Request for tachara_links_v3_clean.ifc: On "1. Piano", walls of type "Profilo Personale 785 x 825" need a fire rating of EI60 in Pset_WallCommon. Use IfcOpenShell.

First a look at what the model holds.

```python
import ifcopenshell
import ifcopenshell.util.element

model = ifcopenshell.open("tachara_links_v3_clean.ifc")
print(model.schema)
storey = next(s for s in model.by_type("IfcBuildingStorey") if s.Name == "1. Piano")
walls = [e for e in ifcopenshell.util.element.get_decomposition(storey) if e.is_a("IfcWall")]
seen = {}
for e in walls:
    element_type = ifcopenshell.util.element.get_type(e)
    key = (element_type.Name if element_type != e and element_type else None, ifcopenshell.util.element.get_pset(e, "Pset_WallCommon", "FireRating"))
    seen[key] = seen.get(key, 0) + 1
for (name, value), count in sorted(seen.items(), key=str):
    print(count, "x", name, "|", value)
```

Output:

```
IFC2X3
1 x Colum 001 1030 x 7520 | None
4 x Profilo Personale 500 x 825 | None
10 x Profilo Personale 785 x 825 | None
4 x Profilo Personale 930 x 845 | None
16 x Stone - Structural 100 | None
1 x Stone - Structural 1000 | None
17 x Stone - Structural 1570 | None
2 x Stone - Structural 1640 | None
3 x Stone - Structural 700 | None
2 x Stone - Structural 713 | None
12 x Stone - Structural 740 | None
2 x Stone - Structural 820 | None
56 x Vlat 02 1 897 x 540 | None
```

```python
import ifcopenshell
import ifcopenshell.api.pset
import ifcopenshell.util.element

model = ifcopenshell.open("tachara_links_v3_clean.ifc")

storey = next(s for s in model.by_type("IfcBuildingStorey") if s.Name == "1. Piano")
walls = [e for e in ifcopenshell.util.element.get_decomposition(storey) if e.is_a("IfcWall")]

count = 0
for e in walls:
    element_type = ifcopenshell.util.element.get_type(e)
    if element_type in (None, e) or element_type.Name != "Profilo Personale 785 x 825":
        continue
    # add_pset returns the element's existing set when there is one.
    pset = ifcopenshell.api.pset.add_pset(model, product=e, name="Pset_WallCommon")
    ifcopenshell.api.pset.edit_pset(model, pset=pset, properties={"FireRating": "EI60"})
    count += 1

print(count, "walls updated")

model.write("tachara_links_v3_clean-out.ifc")
```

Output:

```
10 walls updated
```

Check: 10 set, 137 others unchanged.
